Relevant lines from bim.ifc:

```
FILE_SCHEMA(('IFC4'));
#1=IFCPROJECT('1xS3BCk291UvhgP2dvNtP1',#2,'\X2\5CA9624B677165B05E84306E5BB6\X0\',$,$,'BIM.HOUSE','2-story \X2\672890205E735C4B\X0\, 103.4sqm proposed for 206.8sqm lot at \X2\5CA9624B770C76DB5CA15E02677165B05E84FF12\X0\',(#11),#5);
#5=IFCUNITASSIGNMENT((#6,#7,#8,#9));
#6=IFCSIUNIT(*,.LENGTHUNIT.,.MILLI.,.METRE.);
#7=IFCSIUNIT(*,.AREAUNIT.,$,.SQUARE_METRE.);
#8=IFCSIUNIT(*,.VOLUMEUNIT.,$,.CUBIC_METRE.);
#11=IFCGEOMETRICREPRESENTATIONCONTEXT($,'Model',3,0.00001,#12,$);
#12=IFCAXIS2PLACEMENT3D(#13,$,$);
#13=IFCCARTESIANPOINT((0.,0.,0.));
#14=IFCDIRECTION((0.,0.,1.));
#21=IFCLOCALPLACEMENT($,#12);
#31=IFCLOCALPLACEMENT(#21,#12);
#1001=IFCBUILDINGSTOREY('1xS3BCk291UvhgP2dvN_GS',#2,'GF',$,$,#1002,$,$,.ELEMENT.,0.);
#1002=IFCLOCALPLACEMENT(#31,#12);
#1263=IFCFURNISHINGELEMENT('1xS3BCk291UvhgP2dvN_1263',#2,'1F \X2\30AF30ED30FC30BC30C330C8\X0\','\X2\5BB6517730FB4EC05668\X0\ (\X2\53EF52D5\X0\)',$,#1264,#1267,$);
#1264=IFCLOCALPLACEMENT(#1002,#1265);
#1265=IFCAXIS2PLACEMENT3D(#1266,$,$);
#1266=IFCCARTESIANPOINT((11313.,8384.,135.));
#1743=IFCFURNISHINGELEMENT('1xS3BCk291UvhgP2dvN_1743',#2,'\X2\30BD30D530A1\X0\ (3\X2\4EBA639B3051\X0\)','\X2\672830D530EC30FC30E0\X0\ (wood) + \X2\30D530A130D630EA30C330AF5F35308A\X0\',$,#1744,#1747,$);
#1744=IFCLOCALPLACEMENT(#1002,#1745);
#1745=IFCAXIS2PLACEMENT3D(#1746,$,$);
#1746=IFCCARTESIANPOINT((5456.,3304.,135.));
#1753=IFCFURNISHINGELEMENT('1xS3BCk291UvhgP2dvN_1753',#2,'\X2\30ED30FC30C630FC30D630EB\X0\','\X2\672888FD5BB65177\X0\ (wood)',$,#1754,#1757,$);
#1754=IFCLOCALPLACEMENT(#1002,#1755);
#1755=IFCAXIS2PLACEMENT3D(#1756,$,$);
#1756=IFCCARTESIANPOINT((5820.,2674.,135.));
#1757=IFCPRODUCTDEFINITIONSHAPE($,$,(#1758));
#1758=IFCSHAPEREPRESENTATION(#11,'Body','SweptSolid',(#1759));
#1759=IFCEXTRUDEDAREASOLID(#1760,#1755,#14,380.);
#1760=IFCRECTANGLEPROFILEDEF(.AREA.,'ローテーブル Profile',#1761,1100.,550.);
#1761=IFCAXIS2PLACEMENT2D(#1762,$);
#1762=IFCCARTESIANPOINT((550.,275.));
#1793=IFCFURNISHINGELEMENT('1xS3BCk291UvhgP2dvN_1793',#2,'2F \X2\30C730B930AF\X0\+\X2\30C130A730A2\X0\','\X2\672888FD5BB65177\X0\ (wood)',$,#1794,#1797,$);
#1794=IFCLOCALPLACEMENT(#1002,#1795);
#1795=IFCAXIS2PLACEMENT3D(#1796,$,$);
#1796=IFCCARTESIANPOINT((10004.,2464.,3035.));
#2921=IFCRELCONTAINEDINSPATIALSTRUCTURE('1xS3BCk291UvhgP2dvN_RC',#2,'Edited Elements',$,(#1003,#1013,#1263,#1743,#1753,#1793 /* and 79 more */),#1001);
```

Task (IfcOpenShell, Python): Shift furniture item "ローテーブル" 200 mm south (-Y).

```python
import ifcopenshell
import ifcopenshell.api.geometry
import ifcopenshell.util.placement

model = ifcopenshell.open("bim.ifc")

item = model.by_guid("1xS3BCk291UvhgP2dvN_1753")
matrix = ifcopenshell.util.placement.get_local_placement(item.ObjectPlacement)
matrix[1, 3] -= 200.0
ifcopenshell.api.geometry.edit_object_placement(model, product=item, matrix=matrix, is_si=False)

print(ifcopenshell.util.placement.get_local_placement(item.ObjectPlacement).round(3) + 0.0)

model.write("bim_edited.ifc")
```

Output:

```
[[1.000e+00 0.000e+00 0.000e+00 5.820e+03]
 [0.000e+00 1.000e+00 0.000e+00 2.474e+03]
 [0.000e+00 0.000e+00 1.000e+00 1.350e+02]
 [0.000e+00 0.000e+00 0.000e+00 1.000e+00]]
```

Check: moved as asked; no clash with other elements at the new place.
